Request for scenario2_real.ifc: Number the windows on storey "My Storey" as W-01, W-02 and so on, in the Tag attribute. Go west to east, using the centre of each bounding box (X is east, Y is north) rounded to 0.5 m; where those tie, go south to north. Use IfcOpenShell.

First a look at what the model holds.

```python
import ifcopenshell
import ifcopenshell.util.element
import ifcopenshell.util.placement

model = ifcopenshell.open("scenario2_real.ifc")
print(model.schema)
storey = next(s for s in model.by_type("IfcBuildingStorey") if s.Name == "My Storey")
windows = [e for e in ifcopenshell.util.element.get_decomposition(storey) if e.is_a("IfcWindow")]
for e in sorted(windows, key=lambda e: e.id()):
    origin = ifcopenshell.util.placement.get_local_placement(e.ObjectPlacement)[:3, 3]
    print(e.id(), e.Tag, e.Name, origin.round(2) + 0.0, sep=" | ")
```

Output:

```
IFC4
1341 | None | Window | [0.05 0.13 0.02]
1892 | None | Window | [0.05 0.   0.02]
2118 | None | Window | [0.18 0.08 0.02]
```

```python
import ifcopenshell
import ifcopenshell.geom
import ifcopenshell.util.element
import ifcopenshell.util.shape

model = ifcopenshell.open("scenario2_real.ifc")
settings = ifcopenshell.geom.settings()
settings.set("use-world-coords", True)


def centre(element):
    shape = ifcopenshell.geom.create_shape(settings, element)
    return ifcopenshell.util.shape.get_bbox_centroid(shape.geometry)


storey = next(s for s in model.by_type("IfcBuildingStorey") if s.Name == "My Storey")
windows = [e for e in ifcopenshell.util.element.get_decomposition(storey) if e.is_a("IfcWindow")]

# Insertion points can sit at a corner or the storey origin, so sort by the geometry (in metres).
centres = {e: centre(e) for e in windows}
windows.sort(key=lambda e: (round(centres[e][0] / 0.5), centres[e][1]))

for i, e in enumerate(windows, start=1):
    number = f"W-{i:02d}"
    e.Tag = number
    print(e.id(), number)

model.write("scenario2_real_edited.ifc")
```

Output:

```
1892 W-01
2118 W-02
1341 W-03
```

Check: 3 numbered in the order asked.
